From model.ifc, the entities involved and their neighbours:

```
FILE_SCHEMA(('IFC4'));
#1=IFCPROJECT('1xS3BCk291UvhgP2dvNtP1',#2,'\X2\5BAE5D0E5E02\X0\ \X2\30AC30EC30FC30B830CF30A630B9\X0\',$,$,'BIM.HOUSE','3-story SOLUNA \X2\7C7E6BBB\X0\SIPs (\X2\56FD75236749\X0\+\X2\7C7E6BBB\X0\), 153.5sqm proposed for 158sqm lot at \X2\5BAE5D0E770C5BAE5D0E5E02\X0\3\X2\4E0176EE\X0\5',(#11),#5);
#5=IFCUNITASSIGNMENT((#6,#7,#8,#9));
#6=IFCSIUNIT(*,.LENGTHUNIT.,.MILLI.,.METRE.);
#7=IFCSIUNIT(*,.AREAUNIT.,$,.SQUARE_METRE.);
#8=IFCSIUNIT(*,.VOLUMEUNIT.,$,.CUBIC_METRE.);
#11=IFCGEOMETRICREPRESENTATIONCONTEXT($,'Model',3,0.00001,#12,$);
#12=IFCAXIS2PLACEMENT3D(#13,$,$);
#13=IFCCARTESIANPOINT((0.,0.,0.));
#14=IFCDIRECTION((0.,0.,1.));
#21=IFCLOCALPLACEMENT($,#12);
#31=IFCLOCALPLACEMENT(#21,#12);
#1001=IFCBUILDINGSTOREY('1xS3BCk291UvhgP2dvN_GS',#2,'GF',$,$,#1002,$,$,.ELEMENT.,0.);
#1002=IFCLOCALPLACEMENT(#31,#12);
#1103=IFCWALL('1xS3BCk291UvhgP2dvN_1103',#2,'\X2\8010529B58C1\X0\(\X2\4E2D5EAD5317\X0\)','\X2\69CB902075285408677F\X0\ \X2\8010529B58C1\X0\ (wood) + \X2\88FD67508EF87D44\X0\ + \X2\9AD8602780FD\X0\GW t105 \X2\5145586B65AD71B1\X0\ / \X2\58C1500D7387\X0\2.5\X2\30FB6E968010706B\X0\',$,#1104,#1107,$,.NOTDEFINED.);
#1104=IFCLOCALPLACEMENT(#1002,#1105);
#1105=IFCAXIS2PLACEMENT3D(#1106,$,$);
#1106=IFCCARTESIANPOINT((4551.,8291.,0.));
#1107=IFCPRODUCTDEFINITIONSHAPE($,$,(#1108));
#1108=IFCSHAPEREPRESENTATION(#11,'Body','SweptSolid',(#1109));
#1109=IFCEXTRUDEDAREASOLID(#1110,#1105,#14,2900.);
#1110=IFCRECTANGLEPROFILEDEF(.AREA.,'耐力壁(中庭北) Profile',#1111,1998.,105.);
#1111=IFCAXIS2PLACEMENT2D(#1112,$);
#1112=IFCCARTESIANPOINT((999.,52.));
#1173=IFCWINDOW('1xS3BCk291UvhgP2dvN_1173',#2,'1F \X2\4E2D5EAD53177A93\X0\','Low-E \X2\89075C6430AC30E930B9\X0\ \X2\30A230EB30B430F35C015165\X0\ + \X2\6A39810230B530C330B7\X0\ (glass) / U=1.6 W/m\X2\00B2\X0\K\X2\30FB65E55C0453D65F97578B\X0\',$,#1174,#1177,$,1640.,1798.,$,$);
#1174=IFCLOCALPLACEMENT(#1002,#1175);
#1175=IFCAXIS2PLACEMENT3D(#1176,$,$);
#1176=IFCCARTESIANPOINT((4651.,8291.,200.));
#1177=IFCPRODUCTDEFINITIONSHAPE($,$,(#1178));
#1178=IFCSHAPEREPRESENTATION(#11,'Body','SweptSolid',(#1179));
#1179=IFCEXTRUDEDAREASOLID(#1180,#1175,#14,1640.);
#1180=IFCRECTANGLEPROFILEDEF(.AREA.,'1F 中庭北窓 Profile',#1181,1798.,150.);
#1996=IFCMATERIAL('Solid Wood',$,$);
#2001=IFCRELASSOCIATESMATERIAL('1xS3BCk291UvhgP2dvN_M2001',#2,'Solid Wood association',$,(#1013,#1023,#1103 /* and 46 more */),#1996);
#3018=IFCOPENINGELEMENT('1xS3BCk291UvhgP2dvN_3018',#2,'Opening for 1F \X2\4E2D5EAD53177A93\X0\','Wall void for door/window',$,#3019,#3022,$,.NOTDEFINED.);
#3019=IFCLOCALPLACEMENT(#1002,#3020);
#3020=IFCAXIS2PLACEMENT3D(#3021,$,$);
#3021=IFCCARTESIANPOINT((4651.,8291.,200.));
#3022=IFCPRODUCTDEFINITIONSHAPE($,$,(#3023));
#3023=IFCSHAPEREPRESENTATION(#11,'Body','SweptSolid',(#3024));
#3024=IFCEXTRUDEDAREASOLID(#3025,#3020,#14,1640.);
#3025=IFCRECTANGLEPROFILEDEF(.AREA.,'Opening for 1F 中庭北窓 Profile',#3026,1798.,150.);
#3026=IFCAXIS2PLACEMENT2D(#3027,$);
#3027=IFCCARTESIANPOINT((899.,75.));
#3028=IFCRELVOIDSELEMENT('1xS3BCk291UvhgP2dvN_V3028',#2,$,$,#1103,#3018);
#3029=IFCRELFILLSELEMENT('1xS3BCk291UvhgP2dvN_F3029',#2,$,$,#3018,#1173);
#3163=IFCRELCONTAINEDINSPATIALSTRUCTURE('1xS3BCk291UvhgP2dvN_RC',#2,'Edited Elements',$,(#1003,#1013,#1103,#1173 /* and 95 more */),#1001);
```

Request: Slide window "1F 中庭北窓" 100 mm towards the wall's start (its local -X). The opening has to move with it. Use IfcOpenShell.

```python
import ifcopenshell
import ifcopenshell.api.geometry
import ifcopenshell.util.placement

model = ifcopenshell.open("model.ifc")

window = model.by_guid("1xS3BCk291UvhgP2dvN_1173")
opening = window.FillsVoids[0].RelatingOpeningElement
wall = opening.VoidsElements[0].RelatingBuildingElement

wall_matrix = ifcopenshell.util.placement.get_local_placement(wall.ObjectPlacement)
shift = wall_matrix[:3, 0] * -100.0
before = ifcopenshell.util.placement.get_local_placement(window.ObjectPlacement)[:3, 3].copy()

# The window is not placed relative to its opening, so move both.
for product in (opening, window):
    matrix = ifcopenshell.util.placement.get_local_placement(product.ObjectPlacement)
    matrix[:3, 3] += shift
    ifcopenshell.api.geometry.edit_object_placement(model, product=product, matrix=matrix, is_si=False)

after = ifcopenshell.util.placement.get_local_placement(window.ObjectPlacement)[:3, 3]
print("window moved by", (after - before).round(3) + 0.0)

model.write("model_edited.ifc")
```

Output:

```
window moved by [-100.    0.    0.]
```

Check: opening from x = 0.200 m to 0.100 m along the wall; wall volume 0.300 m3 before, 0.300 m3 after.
